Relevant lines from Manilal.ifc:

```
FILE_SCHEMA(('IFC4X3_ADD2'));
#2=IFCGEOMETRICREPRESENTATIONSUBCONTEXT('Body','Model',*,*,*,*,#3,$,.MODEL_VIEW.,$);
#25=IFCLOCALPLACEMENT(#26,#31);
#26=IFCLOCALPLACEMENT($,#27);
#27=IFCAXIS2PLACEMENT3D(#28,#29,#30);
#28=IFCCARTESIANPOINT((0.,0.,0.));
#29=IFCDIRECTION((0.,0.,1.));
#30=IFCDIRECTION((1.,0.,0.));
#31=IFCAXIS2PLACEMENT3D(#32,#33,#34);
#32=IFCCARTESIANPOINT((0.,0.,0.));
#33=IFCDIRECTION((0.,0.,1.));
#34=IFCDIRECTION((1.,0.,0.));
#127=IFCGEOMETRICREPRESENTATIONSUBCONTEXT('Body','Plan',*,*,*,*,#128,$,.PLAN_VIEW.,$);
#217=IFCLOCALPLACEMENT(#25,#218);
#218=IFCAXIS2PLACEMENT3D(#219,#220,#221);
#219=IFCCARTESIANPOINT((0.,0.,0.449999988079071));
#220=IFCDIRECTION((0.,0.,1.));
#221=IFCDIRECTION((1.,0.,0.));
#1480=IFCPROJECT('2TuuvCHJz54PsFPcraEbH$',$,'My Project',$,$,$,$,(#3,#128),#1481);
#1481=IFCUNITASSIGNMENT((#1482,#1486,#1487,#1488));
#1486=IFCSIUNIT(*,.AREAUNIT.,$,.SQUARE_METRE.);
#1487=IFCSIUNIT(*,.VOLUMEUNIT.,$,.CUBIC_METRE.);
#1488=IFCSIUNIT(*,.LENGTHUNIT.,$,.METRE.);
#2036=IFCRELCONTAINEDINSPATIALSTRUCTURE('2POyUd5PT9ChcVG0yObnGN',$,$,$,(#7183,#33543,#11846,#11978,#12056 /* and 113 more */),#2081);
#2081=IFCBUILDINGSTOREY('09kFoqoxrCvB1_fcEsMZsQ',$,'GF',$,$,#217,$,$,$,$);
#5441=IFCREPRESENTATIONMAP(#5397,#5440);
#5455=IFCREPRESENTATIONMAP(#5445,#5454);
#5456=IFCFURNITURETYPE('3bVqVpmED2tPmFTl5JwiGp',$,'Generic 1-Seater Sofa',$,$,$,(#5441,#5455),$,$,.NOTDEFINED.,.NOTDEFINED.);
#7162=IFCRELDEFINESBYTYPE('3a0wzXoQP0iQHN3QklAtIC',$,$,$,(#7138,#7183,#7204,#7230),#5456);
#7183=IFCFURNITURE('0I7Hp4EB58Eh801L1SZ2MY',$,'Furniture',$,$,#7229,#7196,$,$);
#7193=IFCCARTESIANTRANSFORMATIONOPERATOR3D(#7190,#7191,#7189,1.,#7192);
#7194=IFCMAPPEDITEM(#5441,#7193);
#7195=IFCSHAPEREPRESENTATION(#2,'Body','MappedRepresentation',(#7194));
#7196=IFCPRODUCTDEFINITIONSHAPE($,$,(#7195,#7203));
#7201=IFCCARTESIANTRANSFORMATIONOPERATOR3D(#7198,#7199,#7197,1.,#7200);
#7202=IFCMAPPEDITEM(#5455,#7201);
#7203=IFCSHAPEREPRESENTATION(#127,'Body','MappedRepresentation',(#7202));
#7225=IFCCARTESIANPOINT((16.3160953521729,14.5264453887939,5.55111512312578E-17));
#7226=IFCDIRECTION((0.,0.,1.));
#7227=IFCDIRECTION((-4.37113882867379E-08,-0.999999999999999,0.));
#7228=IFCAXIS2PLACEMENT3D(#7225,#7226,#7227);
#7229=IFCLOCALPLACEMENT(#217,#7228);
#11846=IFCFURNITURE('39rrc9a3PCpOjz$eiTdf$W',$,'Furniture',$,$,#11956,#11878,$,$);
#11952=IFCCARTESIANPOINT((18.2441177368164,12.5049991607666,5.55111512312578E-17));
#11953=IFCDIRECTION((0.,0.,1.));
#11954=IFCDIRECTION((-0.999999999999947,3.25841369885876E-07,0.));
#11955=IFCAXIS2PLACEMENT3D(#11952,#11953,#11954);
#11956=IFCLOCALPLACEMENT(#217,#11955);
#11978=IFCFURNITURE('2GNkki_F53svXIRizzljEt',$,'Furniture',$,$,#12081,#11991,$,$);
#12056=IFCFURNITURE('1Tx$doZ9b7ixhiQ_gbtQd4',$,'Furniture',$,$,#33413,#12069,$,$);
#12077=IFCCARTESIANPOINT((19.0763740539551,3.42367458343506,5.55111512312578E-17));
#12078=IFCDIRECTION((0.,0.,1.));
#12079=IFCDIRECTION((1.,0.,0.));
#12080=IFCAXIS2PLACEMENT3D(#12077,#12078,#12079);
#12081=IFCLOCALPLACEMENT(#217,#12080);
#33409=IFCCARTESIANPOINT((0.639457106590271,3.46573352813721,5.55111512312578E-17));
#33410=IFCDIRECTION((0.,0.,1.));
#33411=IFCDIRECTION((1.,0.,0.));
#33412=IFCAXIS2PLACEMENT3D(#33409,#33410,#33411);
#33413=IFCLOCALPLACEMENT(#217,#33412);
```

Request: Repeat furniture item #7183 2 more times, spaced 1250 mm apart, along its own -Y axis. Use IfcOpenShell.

```python
import ifcopenshell
import ifcopenshell.api.geometry
import ifcopenshell.api.root
import ifcopenshell.util.element
import ifcopenshell.util.placement

model = ifcopenshell.open("Manilal.ifc")

source = model.by_id(7183)
base = ifcopenshell.util.placement.get_local_placement(source.ObjectPlacement)
step = -base[:3, 1] * 1.25

for i in range(1, 3):
    copy = ifcopenshell.api.root.copy_class(model, product=source)
    copy.Representation = ifcopenshell.util.element.copy_deep(
        model, source.Representation, exclude=["IfcGeometricRepresentationContext", "IfcRepresentationMap"]
    )
    matrix = base.copy()
    matrix[:3, 3] += i * step
    print("added at", matrix[:3, 3].round(3) + 0.0)
    ifcopenshell.api.geometry.edit_object_placement(model, product=copy, matrix=matrix, is_si=False)

model.write("Manilal_v2.ifc")
```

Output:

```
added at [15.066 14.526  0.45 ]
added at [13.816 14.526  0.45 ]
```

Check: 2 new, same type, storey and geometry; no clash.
